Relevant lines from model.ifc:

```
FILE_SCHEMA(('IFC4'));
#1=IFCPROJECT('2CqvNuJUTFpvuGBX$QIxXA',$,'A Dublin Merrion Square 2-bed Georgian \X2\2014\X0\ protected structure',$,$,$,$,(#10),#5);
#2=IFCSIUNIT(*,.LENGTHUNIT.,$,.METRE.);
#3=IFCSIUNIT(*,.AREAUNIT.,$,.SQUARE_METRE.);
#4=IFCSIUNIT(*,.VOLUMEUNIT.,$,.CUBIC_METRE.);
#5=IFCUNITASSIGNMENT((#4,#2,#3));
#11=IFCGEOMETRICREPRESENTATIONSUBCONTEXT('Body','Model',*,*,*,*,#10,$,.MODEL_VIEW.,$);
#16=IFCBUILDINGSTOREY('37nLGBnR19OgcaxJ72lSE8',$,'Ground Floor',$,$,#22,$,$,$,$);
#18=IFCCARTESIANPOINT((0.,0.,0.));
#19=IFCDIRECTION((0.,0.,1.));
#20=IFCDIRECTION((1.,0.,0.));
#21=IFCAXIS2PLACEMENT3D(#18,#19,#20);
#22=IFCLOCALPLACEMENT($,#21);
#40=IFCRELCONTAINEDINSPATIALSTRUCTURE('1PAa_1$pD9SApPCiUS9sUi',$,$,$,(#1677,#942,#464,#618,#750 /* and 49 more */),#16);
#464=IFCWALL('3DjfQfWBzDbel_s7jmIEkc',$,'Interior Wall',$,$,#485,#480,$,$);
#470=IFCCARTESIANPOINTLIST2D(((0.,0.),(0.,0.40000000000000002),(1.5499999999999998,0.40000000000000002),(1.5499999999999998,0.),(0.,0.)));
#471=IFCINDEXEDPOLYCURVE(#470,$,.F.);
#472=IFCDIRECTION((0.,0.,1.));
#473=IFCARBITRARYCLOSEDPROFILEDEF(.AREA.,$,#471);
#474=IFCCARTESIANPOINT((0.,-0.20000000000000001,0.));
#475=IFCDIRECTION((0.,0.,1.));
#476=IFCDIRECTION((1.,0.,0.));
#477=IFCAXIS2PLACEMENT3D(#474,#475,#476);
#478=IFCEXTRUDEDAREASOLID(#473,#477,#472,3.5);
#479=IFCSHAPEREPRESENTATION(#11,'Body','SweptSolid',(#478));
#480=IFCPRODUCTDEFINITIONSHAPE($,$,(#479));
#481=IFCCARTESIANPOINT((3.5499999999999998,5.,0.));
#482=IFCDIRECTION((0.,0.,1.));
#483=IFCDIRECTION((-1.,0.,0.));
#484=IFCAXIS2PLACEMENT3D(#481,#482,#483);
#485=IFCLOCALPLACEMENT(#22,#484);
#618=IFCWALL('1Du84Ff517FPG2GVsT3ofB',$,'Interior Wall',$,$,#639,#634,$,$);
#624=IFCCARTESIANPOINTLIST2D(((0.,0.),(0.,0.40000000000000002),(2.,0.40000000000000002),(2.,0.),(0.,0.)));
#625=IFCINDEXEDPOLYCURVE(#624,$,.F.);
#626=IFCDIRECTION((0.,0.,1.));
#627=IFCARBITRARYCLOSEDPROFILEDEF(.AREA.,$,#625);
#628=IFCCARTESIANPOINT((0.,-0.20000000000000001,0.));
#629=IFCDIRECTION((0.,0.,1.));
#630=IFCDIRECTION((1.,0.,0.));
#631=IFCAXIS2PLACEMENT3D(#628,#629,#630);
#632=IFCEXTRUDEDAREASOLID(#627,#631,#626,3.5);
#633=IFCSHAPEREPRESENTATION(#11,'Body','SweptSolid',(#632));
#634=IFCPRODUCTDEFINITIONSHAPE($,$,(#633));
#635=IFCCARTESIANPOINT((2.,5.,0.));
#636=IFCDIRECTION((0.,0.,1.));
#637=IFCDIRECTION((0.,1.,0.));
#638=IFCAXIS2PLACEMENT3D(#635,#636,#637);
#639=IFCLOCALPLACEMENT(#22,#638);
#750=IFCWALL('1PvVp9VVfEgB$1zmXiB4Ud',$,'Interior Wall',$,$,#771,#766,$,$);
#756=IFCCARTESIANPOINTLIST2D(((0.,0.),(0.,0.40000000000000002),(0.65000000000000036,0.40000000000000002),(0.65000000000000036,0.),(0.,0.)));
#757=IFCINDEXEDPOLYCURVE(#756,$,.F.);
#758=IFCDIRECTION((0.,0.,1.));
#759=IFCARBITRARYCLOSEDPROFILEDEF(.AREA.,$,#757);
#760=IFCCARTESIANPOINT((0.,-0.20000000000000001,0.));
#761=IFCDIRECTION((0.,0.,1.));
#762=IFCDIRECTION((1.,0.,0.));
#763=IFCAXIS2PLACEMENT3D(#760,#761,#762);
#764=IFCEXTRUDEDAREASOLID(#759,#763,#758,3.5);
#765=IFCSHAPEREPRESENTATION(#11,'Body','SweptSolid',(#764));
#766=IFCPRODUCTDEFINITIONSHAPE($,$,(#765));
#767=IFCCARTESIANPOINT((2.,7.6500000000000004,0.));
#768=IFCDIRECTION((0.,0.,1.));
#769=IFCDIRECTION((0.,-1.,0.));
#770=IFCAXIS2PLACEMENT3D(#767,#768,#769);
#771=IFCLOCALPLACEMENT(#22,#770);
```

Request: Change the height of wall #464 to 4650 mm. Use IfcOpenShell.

```python
import ifcopenshell
import ifcopenshell.geom
import ifcopenshell.util.representation
import ifcopenshell.util.shape
import ifcopenshell.util.unit

model = ifcopenshell.open("model.ifc")
unit_scale = ifcopenshell.util.unit.calculate_unit_scale(model)
settings = ifcopenshell.geom.settings()


def volume(element):
    """Net volume in cubic metres, openings subtracted."""
    shape = ifcopenshell.geom.create_shape(settings, element)
    return ifcopenshell.util.shape.get_volume(shape.geometry)


wall = model.by_guid("3DjfQfWBzDbel_s7jmIEkc")
before = volume(wall)

body = ifcopenshell.util.representation.get_representation(wall, "Model", "Body")
solid = body.Items[0]
old_height = solid.Depth
solid.Depth = 4.65 / unit_scale
after = volume(wall)

print(f"height {old_height:g} -> {solid.Depth:g}, volume {before:.3f} -> {after:.3f} m3")

model.write("model-out.ifc")
```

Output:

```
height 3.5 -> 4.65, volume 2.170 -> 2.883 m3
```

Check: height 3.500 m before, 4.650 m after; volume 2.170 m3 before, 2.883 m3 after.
